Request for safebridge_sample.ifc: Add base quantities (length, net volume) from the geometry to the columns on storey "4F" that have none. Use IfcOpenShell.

First a look at what the model holds.

```python
import ifcopenshell
import ifcopenshell.util.element
import ifcopenshell.util.unit

model = ifcopenshell.open("safebridge_sample.ifc")
print(model.schema)
for unit_type in ("LENGTHUNIT", "AREAUNIT", "VOLUMEUNIT"):
    print(unit_type, ifcopenshell.util.unit.calculate_unit_scale(model, unit_type))
storey = next(s for s in model.by_type("IfcBuildingStorey") if s.Name == "4F")
columns = [e for e in ifcopenshell.util.element.get_decomposition(storey) if e.is_a("IfcColumn")]
for e in sorted(columns, key=lambda e: e.id()):
    print(e.id(), e.is_a(), e.Name, list(ifcopenshell.util.element.get_psets(e, qtos_only=True)), sep=" | ")
```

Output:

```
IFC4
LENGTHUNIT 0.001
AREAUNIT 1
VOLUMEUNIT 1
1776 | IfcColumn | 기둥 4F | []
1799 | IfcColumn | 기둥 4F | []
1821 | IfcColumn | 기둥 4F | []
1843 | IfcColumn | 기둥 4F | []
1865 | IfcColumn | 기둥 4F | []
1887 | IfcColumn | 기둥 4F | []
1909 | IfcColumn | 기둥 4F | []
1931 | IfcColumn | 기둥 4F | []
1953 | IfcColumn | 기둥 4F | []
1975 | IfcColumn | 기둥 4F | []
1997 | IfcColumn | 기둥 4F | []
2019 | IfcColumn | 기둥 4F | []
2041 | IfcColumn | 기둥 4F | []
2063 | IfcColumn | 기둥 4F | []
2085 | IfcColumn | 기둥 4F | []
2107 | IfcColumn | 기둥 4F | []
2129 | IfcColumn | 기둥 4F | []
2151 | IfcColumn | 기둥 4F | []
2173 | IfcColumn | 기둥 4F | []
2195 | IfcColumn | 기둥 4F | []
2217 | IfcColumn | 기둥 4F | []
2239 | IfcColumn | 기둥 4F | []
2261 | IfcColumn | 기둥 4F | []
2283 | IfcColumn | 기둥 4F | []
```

```python
import ifcopenshell
import ifcopenshell.api.pset
import ifcopenshell.geom
import ifcopenshell.util.element
import ifcopenshell.util.shape
import ifcopenshell.util.unit

model = ifcopenshell.open("safebridge_sample.ifc")
unit_scale = ifcopenshell.util.unit.calculate_unit_scale(model)
volume_scale = ifcopenshell.util.unit.calculate_unit_scale(model, "VOLUMEUNIT")
settings = ifcopenshell.geom.settings()

storey = next(s for s in model.by_type("IfcBuildingStorey") if s.Name == "4F")
columns = [e for e in ifcopenshell.util.element.get_decomposition(storey) if e.is_a("IfcColumn")]

for e in sorted(columns, key=lambda e: e.id()):
    if ifcopenshell.util.element.get_psets(e, qtos_only=True, should_inherit=False):
        continue
    # Geometry comes back in metres, in the element's own axes.
    shape = ifcopenshell.geom.create_shape(settings, e)
    values = {
        "Length": ifcopenshell.util.shape.get_z(shape.geometry) / unit_scale,
        "NetVolume": ifcopenshell.util.shape.get_volume(shape.geometry) / volume_scale,
    }
    qto = ifcopenshell.api.pset.add_qto(model, product=e, name="Qto_ColumnBaseQuantities")
    ifcopenshell.api.pset.edit_qto(model, qto=qto, properties=values)
    print(e.id(), {k: round(v, 3) for k, v in values.items()})

model.write("safebridge_sample_updated.ifc")
```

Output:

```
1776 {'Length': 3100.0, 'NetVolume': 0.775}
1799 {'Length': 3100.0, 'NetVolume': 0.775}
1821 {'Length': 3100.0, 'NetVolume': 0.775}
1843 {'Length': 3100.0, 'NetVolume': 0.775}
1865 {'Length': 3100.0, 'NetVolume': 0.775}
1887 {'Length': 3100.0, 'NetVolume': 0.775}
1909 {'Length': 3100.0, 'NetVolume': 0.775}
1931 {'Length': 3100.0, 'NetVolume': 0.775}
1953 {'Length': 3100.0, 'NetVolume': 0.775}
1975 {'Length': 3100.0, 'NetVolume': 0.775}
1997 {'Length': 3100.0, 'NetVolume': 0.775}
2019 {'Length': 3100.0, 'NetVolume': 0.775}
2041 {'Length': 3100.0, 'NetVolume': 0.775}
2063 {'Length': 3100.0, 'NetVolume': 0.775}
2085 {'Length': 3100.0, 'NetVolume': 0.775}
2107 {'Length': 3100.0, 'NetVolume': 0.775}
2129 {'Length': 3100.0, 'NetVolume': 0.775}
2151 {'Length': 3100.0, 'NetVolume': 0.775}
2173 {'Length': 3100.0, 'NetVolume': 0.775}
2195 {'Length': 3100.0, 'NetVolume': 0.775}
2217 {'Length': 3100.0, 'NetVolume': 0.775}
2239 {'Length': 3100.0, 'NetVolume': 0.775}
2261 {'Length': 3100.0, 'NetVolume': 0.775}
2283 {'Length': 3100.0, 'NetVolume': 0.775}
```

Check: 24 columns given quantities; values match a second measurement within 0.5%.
